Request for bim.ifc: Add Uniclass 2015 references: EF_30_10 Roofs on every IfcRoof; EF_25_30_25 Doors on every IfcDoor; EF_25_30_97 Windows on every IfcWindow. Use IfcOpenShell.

First a look at what the model holds.

```python
import ifcopenshell

model = ifcopenshell.open("bim.ifc")
print(model.schema)
print("classifications:", [c.Name for c in model.by_type("IfcClassification")])
for ifc_class in ("IfcDoor", "IfcRoof", "IfcStair", "IfcWall", "IfcWindow"):
    print(ifc_class, len(model.by_type(ifc_class)))
```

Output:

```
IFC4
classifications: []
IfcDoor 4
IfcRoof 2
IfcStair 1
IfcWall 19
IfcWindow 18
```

```python
import ifcopenshell
import ifcopenshell.api.classification

model = ifcopenshell.open("bim.ifc")

system = ifcopenshell.api.classification.add_classification(model, classification="Uniclass 2015")

codes = {
    "IfcRoof": ("EF_30_10", "Roofs"),
    "IfcDoor": ("EF_25_30_25", "Doors"),
    "IfcWindow": ("EF_25_30_97", "Windows"),
}
for ifc_class, (code, name) in codes.items():
    products = model.by_type(ifc_class)
    ifcopenshell.api.classification.add_reference(
        model, products=products, classification=system, identification=code, name=name
    )
    print(code, len(products))

model.write("bim_v2.ifc")
```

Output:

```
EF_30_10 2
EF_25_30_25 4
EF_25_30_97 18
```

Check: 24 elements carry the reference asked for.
